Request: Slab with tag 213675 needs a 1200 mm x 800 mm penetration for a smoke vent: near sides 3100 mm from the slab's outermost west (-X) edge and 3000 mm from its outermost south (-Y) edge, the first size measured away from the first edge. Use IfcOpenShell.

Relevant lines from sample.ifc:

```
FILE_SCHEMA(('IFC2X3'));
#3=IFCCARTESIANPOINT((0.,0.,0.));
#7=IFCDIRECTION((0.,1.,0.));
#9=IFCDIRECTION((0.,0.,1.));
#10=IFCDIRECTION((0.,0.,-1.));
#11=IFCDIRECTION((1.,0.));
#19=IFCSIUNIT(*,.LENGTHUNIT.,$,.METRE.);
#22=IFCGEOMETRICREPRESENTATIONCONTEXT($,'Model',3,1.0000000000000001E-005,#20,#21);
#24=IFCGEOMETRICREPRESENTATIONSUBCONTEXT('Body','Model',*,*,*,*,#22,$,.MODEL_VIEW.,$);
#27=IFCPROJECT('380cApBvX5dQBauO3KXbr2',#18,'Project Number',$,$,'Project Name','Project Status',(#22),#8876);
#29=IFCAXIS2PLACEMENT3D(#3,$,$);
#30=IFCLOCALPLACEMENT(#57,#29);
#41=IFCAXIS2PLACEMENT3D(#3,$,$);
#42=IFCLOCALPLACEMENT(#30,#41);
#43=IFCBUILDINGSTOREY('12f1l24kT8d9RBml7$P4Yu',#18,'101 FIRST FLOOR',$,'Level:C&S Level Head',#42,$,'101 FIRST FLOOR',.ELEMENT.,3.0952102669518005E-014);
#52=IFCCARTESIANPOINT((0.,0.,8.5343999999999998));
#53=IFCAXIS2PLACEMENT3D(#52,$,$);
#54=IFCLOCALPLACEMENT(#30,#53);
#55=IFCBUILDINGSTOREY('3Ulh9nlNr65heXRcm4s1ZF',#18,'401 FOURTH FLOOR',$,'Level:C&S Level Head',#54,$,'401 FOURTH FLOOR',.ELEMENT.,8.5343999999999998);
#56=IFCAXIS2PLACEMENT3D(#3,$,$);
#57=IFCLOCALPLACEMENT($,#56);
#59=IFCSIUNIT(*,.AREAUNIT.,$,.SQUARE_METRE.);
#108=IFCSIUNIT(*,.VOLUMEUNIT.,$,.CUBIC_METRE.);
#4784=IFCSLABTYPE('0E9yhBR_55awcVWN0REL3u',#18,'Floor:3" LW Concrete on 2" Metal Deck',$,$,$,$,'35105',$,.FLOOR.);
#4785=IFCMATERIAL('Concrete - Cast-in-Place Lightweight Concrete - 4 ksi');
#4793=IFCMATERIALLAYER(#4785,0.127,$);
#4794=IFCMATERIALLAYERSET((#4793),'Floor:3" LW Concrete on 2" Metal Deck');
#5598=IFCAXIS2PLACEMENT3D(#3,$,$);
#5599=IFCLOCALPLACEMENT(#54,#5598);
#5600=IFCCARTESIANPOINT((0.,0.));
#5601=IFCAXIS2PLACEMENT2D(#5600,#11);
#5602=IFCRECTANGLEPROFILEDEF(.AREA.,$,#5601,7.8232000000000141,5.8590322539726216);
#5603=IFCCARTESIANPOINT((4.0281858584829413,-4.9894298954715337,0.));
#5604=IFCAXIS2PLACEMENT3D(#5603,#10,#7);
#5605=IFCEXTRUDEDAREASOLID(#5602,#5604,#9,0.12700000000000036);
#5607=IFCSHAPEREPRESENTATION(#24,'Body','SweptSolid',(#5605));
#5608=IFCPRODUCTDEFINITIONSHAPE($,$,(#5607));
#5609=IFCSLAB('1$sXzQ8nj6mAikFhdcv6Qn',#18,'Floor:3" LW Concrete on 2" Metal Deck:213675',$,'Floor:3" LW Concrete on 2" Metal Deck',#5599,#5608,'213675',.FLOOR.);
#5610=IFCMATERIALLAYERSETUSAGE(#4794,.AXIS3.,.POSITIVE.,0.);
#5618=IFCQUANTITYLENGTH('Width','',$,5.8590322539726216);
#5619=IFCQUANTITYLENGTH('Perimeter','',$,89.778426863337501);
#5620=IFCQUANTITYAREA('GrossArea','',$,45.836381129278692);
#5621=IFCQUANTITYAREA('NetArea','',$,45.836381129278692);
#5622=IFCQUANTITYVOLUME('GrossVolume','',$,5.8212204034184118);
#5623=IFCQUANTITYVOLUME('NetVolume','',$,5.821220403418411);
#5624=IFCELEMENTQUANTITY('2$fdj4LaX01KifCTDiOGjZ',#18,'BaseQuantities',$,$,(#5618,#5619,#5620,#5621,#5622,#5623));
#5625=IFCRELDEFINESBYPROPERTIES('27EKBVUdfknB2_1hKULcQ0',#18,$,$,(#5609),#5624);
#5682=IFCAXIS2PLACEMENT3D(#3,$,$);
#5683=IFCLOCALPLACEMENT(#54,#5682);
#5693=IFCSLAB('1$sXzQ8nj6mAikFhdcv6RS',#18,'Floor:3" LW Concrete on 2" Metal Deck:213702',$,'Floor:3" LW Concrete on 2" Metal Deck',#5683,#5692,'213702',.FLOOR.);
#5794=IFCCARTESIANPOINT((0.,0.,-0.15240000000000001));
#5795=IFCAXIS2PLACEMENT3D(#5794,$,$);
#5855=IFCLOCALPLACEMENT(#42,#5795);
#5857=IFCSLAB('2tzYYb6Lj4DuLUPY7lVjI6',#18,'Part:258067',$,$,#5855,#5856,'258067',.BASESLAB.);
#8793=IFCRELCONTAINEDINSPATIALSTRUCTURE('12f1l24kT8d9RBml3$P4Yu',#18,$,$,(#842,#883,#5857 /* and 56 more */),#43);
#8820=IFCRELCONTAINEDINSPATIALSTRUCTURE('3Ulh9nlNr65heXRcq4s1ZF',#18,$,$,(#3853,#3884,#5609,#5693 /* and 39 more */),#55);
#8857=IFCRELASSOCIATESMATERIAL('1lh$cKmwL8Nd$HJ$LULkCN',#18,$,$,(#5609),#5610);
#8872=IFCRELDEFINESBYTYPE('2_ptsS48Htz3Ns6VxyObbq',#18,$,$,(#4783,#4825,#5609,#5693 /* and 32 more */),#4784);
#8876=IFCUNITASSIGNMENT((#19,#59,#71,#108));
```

```python
import numpy as np
import ifcopenshell
import ifcopenshell.api.feature
import ifcopenshell.api.geometry
import ifcopenshell.api.pset
import ifcopenshell.api.root
import ifcopenshell.geom
import ifcopenshell.util.element
import ifcopenshell.util.placement
import ifcopenshell.util.representation
import ifcopenshell.util.shape
import ifcopenshell.util.unit

model = ifcopenshell.open("sample.ifc")
unit_scale = ifcopenshell.util.unit.calculate_unit_scale(model)
area_scale = ifcopenshell.util.unit.calculate_unit_scale(model, "AREAUNIT")
volume_scale = ifcopenshell.util.unit.calculate_unit_scale(model, "VOLUMEUNIT")
settings = ifcopenshell.geom.settings()


def volume(element):
    """Net volume in cubic metres, openings subtracted."""
    shape = ifcopenshell.geom.create_shape(settings, element)
    return ifcopenshell.util.shape.get_volume(shape.geometry)


slab = model.by_id(5609)
before = volume(slab)

# Extent in the slab's own axes, in metres. The edges named are its -X and -Y sides.
slab_shape = ifcopenshell.geom.create_shape(settings, slab)
vertices = ifcopenshell.util.shape.get_vertices(slab_shape.geometry)
x_min, y_min, bottom = vertices.min(axis=0)
top = vertices[:, 2].max()

opening = ifcopenshell.api.root.create_entity(model, ifc_class="IfcOpeningElement", name="Smoke vent opening")
context = ifcopenshell.util.representation.get_context(model, "Model", "Body", "MODEL_VIEW")
width, depth = 1.2, 0.8
outline = [(0.0, 0.0), (width, 0.0), (width, depth), (0.0, depth), (0.0, 0.0)]
# Overshoot both faces by 50 mm so the cut is clean.
shape = ifcopenshell.api.geometry.add_slab_representation(
    model, context=context, depth=top - bottom + 0.1, polyline=outline
)
ifcopenshell.api.geometry.assign_representation(model, product=opening, representation=shape)

matrix = ifcopenshell.util.placement.get_local_placement(slab.ObjectPlacement)
matrix[:, 3] = matrix @ np.append(np.array([x_min + 3.1, y_min + 3, bottom - 0.05]) / unit_scale, 1.0)
ifcopenshell.api.geometry.edit_object_placement(model, product=opening, matrix=matrix, is_si=False)
ifcopenshell.api.feature.add_feature(model, feature=opening, element=slab)

after = volume(slab)

# Update the slab's stored quantities.
qto = model.by_id(ifcopenshell.util.element.get_pset(slab, "BaseQuantities", should_inherit=False)["id"])
ifcopenshell.api.pset.edit_qto(model, qto=qto, properties={
    "NetArea": after / (top - bottom) / area_scale,
    "NetVolume": after / volume_scale,
})

print(f"slab volume {before:.3f} -> {after:.3f} m3")

model.write("sample_v2.ifc")
```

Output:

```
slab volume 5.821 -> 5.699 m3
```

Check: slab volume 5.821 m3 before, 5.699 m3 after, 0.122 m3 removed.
